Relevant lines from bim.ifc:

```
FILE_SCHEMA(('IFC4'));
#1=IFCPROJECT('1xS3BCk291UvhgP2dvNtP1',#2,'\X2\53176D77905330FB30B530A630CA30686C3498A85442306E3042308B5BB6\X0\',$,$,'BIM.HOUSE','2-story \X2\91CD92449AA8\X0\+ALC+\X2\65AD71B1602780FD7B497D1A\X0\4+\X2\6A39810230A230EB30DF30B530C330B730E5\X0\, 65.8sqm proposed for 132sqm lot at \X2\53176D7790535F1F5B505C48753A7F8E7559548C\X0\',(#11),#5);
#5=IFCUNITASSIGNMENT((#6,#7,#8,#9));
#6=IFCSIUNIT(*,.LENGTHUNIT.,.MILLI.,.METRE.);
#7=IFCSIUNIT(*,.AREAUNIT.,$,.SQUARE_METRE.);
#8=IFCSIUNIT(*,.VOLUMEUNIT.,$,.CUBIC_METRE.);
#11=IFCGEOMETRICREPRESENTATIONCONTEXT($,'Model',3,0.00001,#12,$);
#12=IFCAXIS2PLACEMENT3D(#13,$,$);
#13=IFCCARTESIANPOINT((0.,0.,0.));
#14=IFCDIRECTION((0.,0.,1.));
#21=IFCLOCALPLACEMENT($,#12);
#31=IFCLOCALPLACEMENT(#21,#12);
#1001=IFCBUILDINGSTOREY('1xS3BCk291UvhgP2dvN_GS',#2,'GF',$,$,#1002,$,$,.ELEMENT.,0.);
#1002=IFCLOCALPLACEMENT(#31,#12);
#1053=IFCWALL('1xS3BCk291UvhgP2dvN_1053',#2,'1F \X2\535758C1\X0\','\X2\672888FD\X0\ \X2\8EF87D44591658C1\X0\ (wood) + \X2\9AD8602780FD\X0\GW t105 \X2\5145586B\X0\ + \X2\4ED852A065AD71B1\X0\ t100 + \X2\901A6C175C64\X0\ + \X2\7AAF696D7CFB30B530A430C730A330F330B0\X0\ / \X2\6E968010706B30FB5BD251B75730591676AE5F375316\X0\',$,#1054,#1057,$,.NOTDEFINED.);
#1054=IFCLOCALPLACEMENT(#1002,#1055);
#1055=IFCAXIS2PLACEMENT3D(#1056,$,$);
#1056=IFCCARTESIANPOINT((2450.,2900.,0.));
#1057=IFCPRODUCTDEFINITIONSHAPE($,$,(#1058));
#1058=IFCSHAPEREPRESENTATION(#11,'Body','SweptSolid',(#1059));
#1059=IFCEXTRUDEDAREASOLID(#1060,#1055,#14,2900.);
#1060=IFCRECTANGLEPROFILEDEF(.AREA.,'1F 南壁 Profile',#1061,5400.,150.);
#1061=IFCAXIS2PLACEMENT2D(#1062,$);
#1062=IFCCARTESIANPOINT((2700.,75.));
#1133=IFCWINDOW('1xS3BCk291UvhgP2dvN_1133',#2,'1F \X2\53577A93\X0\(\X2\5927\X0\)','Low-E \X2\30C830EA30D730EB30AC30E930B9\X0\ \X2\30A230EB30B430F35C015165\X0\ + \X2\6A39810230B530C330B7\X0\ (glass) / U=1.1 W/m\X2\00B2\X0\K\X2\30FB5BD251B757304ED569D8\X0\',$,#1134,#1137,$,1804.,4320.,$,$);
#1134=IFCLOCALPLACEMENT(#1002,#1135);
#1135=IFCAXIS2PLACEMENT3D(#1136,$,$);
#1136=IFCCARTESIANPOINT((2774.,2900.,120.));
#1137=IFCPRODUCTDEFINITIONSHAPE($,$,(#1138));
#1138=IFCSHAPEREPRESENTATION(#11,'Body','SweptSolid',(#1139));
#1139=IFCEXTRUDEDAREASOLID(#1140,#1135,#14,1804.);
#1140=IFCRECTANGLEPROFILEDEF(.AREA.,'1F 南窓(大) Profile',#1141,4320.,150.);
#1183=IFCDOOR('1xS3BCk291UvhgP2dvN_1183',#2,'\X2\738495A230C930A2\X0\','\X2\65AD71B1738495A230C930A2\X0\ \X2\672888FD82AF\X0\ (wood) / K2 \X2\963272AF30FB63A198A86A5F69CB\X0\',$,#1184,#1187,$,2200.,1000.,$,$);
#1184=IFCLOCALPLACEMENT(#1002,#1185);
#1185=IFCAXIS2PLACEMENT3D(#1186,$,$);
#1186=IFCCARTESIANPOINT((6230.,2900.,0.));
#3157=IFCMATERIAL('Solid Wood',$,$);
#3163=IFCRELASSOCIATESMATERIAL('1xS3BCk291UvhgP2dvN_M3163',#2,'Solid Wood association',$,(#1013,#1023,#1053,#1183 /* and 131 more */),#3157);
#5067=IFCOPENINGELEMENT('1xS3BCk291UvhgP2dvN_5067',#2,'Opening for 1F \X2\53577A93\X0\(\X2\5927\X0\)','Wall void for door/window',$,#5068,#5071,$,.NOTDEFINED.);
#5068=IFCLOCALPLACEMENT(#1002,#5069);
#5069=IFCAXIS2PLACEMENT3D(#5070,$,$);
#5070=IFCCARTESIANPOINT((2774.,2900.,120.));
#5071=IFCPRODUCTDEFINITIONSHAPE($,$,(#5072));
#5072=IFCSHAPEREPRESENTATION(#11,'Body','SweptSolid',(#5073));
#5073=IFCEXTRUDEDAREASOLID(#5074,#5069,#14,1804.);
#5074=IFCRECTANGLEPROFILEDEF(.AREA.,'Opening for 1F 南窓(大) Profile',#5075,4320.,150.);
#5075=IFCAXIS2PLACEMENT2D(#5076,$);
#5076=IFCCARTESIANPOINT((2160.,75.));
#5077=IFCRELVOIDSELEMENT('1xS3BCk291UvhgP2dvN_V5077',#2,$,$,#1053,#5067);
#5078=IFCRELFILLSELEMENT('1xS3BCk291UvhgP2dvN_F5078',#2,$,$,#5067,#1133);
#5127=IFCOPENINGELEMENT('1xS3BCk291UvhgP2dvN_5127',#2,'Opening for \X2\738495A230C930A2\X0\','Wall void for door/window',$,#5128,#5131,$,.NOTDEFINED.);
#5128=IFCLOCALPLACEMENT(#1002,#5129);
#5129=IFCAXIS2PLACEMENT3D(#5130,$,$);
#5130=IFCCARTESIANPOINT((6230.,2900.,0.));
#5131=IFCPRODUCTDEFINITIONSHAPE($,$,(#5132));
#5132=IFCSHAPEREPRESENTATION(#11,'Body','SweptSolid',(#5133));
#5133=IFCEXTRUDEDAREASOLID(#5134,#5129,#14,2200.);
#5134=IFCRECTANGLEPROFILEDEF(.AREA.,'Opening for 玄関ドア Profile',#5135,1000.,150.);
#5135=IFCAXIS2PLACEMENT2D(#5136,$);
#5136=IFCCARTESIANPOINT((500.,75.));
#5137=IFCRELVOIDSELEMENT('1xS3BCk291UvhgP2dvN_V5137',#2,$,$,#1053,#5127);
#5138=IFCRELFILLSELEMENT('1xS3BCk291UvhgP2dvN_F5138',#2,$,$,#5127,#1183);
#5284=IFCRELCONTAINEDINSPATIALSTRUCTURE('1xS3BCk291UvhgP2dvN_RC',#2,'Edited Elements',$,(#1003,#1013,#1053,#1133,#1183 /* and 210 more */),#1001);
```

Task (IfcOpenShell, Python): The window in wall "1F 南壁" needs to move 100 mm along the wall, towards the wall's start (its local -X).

```python
import ifcopenshell
import ifcopenshell.api.geometry
import ifcopenshell.util.placement
import ifcopenshell.util.unit

model = ifcopenshell.open("bim.ifc")
unit_scale = ifcopenshell.util.unit.calculate_unit_scale(model)

window = model.by_id(1133)
opening = window.FillsVoids[0].RelatingOpeningElement
wall = opening.VoidsElements[0].RelatingBuildingElement

wall_matrix = ifcopenshell.util.placement.get_local_placement(wall.ObjectPlacement)
shift = wall_matrix[:3, 0] * -0.1 / unit_scale
before = ifcopenshell.util.placement.get_local_placement(window.ObjectPlacement)[:3, 3].copy()

# The window is not placed relative to its opening, so move both.
for product in (opening, window):
    matrix = ifcopenshell.util.placement.get_local_placement(product.ObjectPlacement)
    matrix[:3, 3] += shift
    ifcopenshell.api.geometry.edit_object_placement(model, product=product, matrix=matrix, is_si=False)

after = ifcopenshell.util.placement.get_local_placement(window.ObjectPlacement)[:3, 3]
print("window moved by", (after - before).round(3) + 0.0)

model.write("bim_edited.ifc")
```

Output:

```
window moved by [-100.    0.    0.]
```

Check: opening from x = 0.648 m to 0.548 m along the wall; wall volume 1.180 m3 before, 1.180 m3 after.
